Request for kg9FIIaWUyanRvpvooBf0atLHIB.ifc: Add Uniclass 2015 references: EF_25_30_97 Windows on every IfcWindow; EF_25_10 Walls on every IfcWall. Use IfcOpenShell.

First a look at what the model holds.

```python
import ifcopenshell

model = ifcopenshell.open("kg9FIIaWUyanRvpvooBf0atLHIB.ifc")
print(model.schema)
print("classifications:", [c.Name for c in model.by_type("IfcClassification")])
for ifc_class in ("IfcDoor", "IfcRoof", "IfcStair", "IfcWall", "IfcWindow"):
    print(ifc_class, len(model.by_type(ifc_class)))
```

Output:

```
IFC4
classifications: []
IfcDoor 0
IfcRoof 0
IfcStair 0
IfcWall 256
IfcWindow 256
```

```python
import ifcopenshell
import ifcopenshell.api.classification

model = ifcopenshell.open("kg9FIIaWUyanRvpvooBf0atLHIB.ifc")

system = ifcopenshell.api.classification.add_classification(model, classification="Uniclass 2015")

codes = {
    "IfcWindow": ("EF_25_30_97", "Windows"),
    "IfcWall": ("EF_25_10", "Walls"),
}
for ifc_class, (code, name) in codes.items():
    products = model.by_type(ifc_class)
    ifcopenshell.api.classification.add_reference(
        model, products=products, classification=system, identification=code, name=name
    )
    print(code, len(products))

model.write("kg9FIIaWUyanRvpvooBf0atLHIB_edited.ifc")
```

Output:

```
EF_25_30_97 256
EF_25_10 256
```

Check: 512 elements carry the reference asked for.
